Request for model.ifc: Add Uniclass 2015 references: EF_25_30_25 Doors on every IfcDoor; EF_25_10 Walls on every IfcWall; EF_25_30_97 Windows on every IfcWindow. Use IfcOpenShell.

First a look at what the model holds.

```python
import ifcopenshell

model = ifcopenshell.open("model.ifc")
print(model.schema)
print("classifications:", [c.Name for c in model.by_type("IfcClassification")])
for ifc_class in ("IfcDoor", "IfcRoof", "IfcStair", "IfcWall", "IfcWindow"):
    print(ifc_class, len(model.by_type(ifc_class)))
```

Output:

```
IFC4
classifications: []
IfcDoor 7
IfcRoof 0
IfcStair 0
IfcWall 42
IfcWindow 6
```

```python
import ifcopenshell
import ifcopenshell.api.classification

model = ifcopenshell.open("model.ifc")

system = ifcopenshell.api.classification.add_classification(model, classification="Uniclass 2015")

codes = {
    "IfcDoor": ("EF_25_30_25", "Doors"),
    "IfcWall": ("EF_25_10", "Walls"),
    "IfcWindow": ("EF_25_30_97", "Windows"),
}
for ifc_class, (code, name) in codes.items():
    products = model.by_type(ifc_class)
    ifcopenshell.api.classification.add_reference(
        model, products=products, classification=system, identification=code, name=name
    )
    print(code, len(products))

model.write("model_updated.ifc")
```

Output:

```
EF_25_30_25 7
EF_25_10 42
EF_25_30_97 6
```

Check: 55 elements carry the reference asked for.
